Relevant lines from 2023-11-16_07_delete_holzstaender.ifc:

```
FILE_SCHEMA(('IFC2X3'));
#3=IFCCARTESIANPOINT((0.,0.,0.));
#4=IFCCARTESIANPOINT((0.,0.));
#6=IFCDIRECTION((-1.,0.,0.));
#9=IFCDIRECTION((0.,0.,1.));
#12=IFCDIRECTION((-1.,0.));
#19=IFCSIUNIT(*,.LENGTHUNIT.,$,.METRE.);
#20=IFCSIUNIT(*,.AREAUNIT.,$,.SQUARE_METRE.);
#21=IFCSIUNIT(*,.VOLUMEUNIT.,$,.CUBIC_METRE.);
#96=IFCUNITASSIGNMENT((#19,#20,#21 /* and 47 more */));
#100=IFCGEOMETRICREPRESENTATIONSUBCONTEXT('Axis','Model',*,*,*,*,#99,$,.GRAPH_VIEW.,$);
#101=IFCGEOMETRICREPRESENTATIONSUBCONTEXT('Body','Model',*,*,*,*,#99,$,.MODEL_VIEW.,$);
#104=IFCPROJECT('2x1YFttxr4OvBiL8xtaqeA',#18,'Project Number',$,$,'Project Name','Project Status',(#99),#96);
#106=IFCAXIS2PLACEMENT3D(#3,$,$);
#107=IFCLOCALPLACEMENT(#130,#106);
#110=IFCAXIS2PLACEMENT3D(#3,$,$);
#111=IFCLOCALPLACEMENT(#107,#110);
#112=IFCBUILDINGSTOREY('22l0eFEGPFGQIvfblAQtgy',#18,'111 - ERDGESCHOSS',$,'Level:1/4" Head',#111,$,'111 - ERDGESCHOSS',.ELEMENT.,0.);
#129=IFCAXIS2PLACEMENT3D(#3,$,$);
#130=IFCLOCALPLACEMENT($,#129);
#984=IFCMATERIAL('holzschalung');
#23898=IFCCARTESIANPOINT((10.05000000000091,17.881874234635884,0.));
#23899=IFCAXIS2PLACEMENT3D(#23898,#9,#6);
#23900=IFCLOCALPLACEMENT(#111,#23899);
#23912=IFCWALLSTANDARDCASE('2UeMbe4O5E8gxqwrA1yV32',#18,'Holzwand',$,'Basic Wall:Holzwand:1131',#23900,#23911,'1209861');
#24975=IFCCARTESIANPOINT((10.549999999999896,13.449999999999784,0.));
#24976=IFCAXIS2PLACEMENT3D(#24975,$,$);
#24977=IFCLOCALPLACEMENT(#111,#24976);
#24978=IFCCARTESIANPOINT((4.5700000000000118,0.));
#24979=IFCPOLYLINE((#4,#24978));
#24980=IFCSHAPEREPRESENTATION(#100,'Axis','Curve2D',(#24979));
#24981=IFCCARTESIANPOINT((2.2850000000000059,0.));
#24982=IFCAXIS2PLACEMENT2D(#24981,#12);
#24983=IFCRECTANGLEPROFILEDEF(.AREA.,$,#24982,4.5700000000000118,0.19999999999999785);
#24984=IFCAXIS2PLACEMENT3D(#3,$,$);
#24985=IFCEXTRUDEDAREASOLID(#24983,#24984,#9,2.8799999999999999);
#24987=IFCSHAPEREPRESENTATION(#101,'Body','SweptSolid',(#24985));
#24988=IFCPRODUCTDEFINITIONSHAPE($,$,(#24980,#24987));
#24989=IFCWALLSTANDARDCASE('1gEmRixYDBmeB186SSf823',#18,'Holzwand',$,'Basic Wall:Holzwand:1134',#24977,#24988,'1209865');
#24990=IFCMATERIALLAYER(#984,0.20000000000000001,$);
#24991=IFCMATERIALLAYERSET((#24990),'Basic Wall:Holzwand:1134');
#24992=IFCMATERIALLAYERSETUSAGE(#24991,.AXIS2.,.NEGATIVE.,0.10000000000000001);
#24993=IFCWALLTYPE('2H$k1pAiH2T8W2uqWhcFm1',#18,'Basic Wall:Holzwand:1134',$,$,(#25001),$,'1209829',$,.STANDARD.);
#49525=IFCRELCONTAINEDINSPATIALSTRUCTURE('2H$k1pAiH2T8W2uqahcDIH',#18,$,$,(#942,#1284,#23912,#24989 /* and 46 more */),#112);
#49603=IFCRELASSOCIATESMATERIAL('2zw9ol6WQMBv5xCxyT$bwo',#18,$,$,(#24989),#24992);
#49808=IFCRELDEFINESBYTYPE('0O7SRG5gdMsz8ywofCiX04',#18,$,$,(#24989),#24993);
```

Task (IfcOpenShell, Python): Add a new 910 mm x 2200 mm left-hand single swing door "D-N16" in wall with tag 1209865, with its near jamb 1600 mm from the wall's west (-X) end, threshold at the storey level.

```python
import numpy as np
import ifcopenshell
import ifcopenshell.api.feature
import ifcopenshell.api.geometry
import ifcopenshell.api.root
import ifcopenshell.api.spatial
import ifcopenshell.api.type
import ifcopenshell.geom
import ifcopenshell.util.element
import ifcopenshell.util.placement
import ifcopenshell.util.representation
import ifcopenshell.util.shape
import ifcopenshell.util.unit

model = ifcopenshell.open("2023-11-16_07_delete_holzstaender.ifc")
unit_scale = ifcopenshell.util.unit.calculate_unit_scale(model)
settings = ifcopenshell.geom.settings()


def volume(element):
    """Net volume in cubic metres, openings subtracted."""
    shape = ifcopenshell.geom.create_shape(settings, element)
    return ifcopenshell.util.shape.get_volume(shape.geometry)


wall = model.by_id(24989)
storey = ifcopenshell.util.element.get_container(wall, ifc_class="IfcBuildingStorey")
context = ifcopenshell.util.representation.get_context(model, "Model", "Body", "MODEL_VIEW")
before = volume(wall)

width, height, from_end, sill = 0.91, 2.2, 1.6, 0.0  # metres

# The wall runs along its own X axis, and the end named is its -X end.
wall_shape = ifcopenshell.geom.create_shape(settings, wall)
x, y, z = ifcopenshell.util.shape.get_vertices(wall_shape.geometry).T
start = x.min() + from_end
face, thickness = float(y.min()), float(y.max() - y.min())
wall_matrix = ifcopenshell.util.placement.get_local_placement(wall.ObjectPlacement)
level = ifcopenshell.util.placement.get_local_placement(storey.ObjectPlacement)[2, 3]


def in_wall(x, y):
    """Placement at x, y metres in the wall's axes, at sill height."""
    matrix = wall_matrix.copy()
    matrix[:, 3] = wall_matrix @ np.array([x / unit_scale, y / unit_scale, 0.0, 1.0])
    matrix[2, 3] = level + sill / unit_scale
    return matrix


# Opening: a box that overshoots both wall faces by 50 mm.
opening = ifcopenshell.api.root.create_entity(model, ifc_class="IfcOpeningElement")
box = ifcopenshell.api.geometry.add_wall_representation(
    model, context=context, length=width, height=height, thickness=thickness + 0.1
)
ifcopenshell.api.geometry.assign_representation(model, product=opening, representation=box)
ifcopenshell.api.geometry.edit_object_placement(model, product=opening, matrix=in_wall(start, face - 0.05), is_si=False)
ifcopenshell.api.feature.add_feature(model, feature=opening, element=wall)

door = ifcopenshell.api.root.create_entity(model, ifc_class="IfcDoor", name="D-N16")
door.OverallWidth, door.OverallHeight = width / unit_scale, height / unit_scale
body = ifcopenshell.api.geometry.add_door_representation(
    model,
    context=context,
    overall_width=door.OverallWidth,
    overall_height=door.OverallHeight,
    operation_type="SINGLE_SWING_LEFT",
    lining_properties={"LiningDepth": thickness / unit_scale, "ThresholdDepth": thickness / unit_scale},
)
ifcopenshell.api.geometry.assign_representation(model, product=door, representation=body)
ifcopenshell.api.spatial.assign_container(model, products=[door], relating_structure=storey)
fills = ifcopenshell.api.feature.add_filling(model, opening=opening, element=door)
fills.OwnerHistory = door.OwnerHistory  # required in IFC2X3

# IFC2X3 keeps the operation on the door style.
style = ifcopenshell.api.root.create_entity(model, ifc_class="IfcDoorStyle", name="D-N16")
style.OperationType, style.ConstructionType = "SINGLE_SWING_LEFT", "NOTDEFINED"
style.ParameterTakesPrecedence = style.Sizeable = False
ifcopenshell.api.type.assign_type(model, related_objects=[door], relating_type=style)

# The lining spans the wall, so the door starts at the wall face.
ifcopenshell.api.geometry.edit_object_placement(model, product=door, matrix=in_wall(start, face), is_si=False)

after = volume(wall)

print(f"wall volume {before:.3f} -> {after:.3f} m3")

model.write("2023-11-16_07_delete_holzstaender-out.ifc")
```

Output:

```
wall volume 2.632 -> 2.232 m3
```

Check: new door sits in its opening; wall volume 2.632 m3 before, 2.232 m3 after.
